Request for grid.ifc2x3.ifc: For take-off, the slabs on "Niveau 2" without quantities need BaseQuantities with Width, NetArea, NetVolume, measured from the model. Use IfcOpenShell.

First a look at what the model holds.

```python
import ifcopenshell
import ifcopenshell.util.element
import ifcopenshell.util.unit

model = ifcopenshell.open("grid.ifc2x3.ifc")
print(model.schema)
for unit_type in ("LENGTHUNIT", "AREAUNIT", "VOLUMEUNIT"):
    print(unit_type, ifcopenshell.util.unit.calculate_unit_scale(model, unit_type))
storey = next(s for s in model.by_type("IfcBuildingStorey") if s.Name == "Niveau 2")
slabs = [e for e in ifcopenshell.util.element.get_decomposition(storey) if e.is_a("IfcSlab")]
for e in sorted(slabs, key=lambda e: e.id()):
    print(e.id(), e.is_a(), e.Name, list(ifcopenshell.util.element.get_psets(e, qtos_only=True)), sep=" | ")
```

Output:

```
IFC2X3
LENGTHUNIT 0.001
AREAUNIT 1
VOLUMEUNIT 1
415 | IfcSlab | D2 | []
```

```python
import ifcopenshell
import ifcopenshell.api.pset
import ifcopenshell.geom
import ifcopenshell.util.element
import ifcopenshell.util.shape
import ifcopenshell.util.unit

model = ifcopenshell.open("grid.ifc2x3.ifc")
unit_scale = ifcopenshell.util.unit.calculate_unit_scale(model)
area_scale = ifcopenshell.util.unit.calculate_unit_scale(model, "AREAUNIT")
volume_scale = ifcopenshell.util.unit.calculate_unit_scale(model, "VOLUMEUNIT")
settings = ifcopenshell.geom.settings()

storey = next(s for s in model.by_type("IfcBuildingStorey") if s.Name == "Niveau 2")
slabs = [e for e in ifcopenshell.util.element.get_decomposition(storey) if e.is_a("IfcSlab")]

for e in sorted(slabs, key=lambda e: e.id()):
    if ifcopenshell.util.element.get_psets(e, qtos_only=True, should_inherit=False):
        continue
    # Geometry comes back in metres, in the element's own axes.
    shape = ifcopenshell.geom.create_shape(settings, e)
    values = {
        "Width": ifcopenshell.util.shape.get_z(shape.geometry) / unit_scale,
        "NetArea": ifcopenshell.util.shape.get_footprint_area(shape.geometry) / area_scale,
        "NetVolume": ifcopenshell.util.shape.get_volume(shape.geometry) / volume_scale,
    }
    qto = ifcopenshell.api.pset.add_qto(model, product=e, name="BaseQuantities")
    ifcopenshell.api.pset.edit_qto(model, qto=qto, properties=values)
    print(e.id(), {k: round(v, 3) for k, v in values.items()})

model.write("grid.ifc2x3-out.ifc")
```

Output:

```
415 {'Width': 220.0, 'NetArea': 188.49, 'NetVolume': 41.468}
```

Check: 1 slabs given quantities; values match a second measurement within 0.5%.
